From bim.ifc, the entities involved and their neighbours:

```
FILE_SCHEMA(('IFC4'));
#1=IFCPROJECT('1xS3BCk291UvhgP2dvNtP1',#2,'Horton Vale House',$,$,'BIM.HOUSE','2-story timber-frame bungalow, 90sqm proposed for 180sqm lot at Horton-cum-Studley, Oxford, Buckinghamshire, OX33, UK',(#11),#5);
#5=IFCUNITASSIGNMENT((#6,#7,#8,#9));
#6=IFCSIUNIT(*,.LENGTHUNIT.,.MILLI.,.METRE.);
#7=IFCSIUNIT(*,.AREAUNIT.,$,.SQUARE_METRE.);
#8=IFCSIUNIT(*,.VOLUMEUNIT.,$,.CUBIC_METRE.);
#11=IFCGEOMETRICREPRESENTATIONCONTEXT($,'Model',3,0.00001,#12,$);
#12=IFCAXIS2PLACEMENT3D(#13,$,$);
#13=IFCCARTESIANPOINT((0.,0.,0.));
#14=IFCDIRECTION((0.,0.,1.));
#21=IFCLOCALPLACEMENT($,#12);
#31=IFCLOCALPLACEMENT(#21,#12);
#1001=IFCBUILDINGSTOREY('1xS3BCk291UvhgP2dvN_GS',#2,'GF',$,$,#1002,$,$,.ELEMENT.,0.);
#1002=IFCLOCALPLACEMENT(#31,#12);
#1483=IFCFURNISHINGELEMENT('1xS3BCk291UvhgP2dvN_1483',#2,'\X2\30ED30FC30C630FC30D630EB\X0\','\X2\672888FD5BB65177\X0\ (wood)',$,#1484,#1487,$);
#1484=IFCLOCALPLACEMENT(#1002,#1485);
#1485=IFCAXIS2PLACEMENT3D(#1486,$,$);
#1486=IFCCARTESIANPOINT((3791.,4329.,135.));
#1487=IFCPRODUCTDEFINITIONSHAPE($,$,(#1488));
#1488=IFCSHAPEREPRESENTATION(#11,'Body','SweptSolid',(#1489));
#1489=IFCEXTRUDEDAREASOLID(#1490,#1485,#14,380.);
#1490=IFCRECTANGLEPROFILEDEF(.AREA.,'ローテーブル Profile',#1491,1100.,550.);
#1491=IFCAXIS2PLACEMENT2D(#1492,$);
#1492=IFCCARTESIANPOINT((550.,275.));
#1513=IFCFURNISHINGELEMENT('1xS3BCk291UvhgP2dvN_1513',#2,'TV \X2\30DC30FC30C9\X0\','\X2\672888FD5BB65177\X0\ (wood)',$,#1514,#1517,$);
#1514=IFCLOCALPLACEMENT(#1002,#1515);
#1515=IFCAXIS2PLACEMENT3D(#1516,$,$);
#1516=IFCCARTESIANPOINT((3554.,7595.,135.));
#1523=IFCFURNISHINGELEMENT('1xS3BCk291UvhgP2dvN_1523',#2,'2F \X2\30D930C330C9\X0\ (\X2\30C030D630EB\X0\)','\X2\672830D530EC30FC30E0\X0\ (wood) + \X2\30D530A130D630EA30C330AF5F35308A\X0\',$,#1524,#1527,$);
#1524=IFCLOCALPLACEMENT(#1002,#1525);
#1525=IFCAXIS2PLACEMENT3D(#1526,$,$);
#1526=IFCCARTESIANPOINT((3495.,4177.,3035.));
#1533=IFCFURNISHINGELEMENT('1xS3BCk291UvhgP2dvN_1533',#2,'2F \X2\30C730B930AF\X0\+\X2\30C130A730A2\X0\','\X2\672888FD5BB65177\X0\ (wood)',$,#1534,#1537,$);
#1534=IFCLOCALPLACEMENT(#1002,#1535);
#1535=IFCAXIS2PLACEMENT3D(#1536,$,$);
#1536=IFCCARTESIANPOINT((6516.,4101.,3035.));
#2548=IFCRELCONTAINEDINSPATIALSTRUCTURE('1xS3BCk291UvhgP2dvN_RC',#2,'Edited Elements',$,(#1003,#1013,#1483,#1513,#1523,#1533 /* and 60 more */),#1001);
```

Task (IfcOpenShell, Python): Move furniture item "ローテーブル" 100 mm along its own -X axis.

```python
import ifcopenshell
import ifcopenshell.api.geometry
import ifcopenshell.util.placement

model = ifcopenshell.open("bim.ifc")

item = model.by_guid("1xS3BCk291UvhgP2dvN_1483")
matrix = ifcopenshell.util.placement.get_local_placement(item.ObjectPlacement)
matrix[:3, 3] -= matrix[:3, 0] * 100.0
ifcopenshell.api.geometry.edit_object_placement(model, product=item, matrix=matrix, is_si=False)

print(ifcopenshell.util.placement.get_local_placement(item.ObjectPlacement).round(3) + 0.0)

model.write("bim_edited.ifc")
```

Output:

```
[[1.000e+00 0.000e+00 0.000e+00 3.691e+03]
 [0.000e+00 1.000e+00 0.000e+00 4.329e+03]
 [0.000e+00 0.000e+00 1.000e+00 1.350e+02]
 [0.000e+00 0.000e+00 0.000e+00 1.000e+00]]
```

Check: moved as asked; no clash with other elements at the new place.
